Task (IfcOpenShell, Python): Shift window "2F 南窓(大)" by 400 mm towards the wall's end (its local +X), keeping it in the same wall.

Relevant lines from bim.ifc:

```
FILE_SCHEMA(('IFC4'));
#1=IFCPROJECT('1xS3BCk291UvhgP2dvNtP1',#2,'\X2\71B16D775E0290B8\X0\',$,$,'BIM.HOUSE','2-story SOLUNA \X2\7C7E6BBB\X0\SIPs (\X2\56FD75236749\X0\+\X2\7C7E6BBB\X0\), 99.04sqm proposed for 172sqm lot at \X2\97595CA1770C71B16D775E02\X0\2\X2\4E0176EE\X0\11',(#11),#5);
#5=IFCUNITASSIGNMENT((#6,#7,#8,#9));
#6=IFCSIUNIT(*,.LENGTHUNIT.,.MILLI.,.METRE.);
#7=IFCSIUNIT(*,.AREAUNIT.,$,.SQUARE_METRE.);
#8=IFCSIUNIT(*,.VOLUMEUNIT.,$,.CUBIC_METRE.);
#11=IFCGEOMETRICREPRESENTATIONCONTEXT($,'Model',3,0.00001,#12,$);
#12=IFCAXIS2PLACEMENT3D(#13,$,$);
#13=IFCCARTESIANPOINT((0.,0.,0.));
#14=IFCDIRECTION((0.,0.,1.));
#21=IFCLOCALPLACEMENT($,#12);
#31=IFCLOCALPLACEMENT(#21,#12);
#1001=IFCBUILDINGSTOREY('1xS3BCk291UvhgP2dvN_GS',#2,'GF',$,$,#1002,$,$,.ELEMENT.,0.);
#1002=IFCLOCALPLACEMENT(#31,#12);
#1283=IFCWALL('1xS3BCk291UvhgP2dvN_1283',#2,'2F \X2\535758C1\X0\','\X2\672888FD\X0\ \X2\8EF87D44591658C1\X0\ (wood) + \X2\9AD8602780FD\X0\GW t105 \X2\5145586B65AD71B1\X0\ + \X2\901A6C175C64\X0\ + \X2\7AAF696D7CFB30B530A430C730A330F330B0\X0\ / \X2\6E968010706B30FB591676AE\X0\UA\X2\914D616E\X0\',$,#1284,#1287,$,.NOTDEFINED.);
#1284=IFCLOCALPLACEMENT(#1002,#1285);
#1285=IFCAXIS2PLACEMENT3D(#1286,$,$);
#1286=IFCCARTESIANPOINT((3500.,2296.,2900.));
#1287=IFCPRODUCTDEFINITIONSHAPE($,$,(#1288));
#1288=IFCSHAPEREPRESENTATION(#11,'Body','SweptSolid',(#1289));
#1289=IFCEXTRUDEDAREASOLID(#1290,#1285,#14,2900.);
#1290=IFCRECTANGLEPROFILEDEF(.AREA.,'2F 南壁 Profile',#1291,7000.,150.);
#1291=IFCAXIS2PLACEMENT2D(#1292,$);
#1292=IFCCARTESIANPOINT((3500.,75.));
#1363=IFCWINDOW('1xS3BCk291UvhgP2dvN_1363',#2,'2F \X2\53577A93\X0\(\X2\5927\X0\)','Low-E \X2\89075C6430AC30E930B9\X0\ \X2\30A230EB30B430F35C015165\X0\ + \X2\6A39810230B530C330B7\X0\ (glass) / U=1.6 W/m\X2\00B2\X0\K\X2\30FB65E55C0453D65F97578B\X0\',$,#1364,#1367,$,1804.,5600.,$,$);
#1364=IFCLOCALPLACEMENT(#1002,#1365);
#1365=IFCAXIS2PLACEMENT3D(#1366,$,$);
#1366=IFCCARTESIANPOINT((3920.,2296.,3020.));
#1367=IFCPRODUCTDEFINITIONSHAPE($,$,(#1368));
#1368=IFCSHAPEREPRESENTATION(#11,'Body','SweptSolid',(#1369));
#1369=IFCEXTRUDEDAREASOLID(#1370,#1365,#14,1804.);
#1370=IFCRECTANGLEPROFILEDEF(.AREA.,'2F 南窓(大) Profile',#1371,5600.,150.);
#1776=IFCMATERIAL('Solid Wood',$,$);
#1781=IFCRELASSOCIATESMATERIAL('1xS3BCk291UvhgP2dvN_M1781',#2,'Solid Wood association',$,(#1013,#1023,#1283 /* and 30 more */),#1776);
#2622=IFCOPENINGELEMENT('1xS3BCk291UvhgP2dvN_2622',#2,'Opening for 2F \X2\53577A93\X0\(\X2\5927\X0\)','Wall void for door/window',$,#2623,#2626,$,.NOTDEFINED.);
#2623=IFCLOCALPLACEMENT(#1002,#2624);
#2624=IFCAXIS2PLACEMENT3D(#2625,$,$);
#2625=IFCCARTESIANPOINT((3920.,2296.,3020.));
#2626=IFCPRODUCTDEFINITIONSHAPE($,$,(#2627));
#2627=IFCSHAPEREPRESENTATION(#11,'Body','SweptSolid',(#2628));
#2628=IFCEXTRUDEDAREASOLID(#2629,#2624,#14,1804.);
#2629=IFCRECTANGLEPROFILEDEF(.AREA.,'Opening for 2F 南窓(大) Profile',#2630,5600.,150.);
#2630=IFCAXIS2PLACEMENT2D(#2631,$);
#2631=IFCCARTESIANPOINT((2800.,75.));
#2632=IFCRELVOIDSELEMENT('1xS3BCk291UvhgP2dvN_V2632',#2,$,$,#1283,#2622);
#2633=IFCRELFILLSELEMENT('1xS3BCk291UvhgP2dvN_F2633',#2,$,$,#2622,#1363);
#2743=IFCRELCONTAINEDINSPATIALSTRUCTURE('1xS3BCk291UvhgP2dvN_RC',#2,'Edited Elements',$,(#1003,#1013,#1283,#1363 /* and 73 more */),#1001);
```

```python
import ifcopenshell
import ifcopenshell.api.geometry
import ifcopenshell.util.placement

model = ifcopenshell.open("bim.ifc")

window = model.by_guid("1xS3BCk291UvhgP2dvN_1363")
opening = window.FillsVoids[0].RelatingOpeningElement
wall = opening.VoidsElements[0].RelatingBuildingElement

wall_matrix = ifcopenshell.util.placement.get_local_placement(wall.ObjectPlacement)
shift = wall_matrix[:3, 0] * 400.0
before = ifcopenshell.util.placement.get_local_placement(window.ObjectPlacement)[:3, 3].copy()

# The window is not placed relative to its opening, so move both.
for product in (opening, window):
    matrix = ifcopenshell.util.placement.get_local_placement(product.ObjectPlacement)
    matrix[:3, 3] += shift
    ifcopenshell.api.geometry.edit_object_placement(model, product=product, matrix=matrix, is_si=False)

after = ifcopenshell.util.placement.get_local_placement(window.ObjectPlacement)[:3, 3]
print("window moved by", (after - before).round(3) + 0.0)

model.write("bim_v2.ifc")
```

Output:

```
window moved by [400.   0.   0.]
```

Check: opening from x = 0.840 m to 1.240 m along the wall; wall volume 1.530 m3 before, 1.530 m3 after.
